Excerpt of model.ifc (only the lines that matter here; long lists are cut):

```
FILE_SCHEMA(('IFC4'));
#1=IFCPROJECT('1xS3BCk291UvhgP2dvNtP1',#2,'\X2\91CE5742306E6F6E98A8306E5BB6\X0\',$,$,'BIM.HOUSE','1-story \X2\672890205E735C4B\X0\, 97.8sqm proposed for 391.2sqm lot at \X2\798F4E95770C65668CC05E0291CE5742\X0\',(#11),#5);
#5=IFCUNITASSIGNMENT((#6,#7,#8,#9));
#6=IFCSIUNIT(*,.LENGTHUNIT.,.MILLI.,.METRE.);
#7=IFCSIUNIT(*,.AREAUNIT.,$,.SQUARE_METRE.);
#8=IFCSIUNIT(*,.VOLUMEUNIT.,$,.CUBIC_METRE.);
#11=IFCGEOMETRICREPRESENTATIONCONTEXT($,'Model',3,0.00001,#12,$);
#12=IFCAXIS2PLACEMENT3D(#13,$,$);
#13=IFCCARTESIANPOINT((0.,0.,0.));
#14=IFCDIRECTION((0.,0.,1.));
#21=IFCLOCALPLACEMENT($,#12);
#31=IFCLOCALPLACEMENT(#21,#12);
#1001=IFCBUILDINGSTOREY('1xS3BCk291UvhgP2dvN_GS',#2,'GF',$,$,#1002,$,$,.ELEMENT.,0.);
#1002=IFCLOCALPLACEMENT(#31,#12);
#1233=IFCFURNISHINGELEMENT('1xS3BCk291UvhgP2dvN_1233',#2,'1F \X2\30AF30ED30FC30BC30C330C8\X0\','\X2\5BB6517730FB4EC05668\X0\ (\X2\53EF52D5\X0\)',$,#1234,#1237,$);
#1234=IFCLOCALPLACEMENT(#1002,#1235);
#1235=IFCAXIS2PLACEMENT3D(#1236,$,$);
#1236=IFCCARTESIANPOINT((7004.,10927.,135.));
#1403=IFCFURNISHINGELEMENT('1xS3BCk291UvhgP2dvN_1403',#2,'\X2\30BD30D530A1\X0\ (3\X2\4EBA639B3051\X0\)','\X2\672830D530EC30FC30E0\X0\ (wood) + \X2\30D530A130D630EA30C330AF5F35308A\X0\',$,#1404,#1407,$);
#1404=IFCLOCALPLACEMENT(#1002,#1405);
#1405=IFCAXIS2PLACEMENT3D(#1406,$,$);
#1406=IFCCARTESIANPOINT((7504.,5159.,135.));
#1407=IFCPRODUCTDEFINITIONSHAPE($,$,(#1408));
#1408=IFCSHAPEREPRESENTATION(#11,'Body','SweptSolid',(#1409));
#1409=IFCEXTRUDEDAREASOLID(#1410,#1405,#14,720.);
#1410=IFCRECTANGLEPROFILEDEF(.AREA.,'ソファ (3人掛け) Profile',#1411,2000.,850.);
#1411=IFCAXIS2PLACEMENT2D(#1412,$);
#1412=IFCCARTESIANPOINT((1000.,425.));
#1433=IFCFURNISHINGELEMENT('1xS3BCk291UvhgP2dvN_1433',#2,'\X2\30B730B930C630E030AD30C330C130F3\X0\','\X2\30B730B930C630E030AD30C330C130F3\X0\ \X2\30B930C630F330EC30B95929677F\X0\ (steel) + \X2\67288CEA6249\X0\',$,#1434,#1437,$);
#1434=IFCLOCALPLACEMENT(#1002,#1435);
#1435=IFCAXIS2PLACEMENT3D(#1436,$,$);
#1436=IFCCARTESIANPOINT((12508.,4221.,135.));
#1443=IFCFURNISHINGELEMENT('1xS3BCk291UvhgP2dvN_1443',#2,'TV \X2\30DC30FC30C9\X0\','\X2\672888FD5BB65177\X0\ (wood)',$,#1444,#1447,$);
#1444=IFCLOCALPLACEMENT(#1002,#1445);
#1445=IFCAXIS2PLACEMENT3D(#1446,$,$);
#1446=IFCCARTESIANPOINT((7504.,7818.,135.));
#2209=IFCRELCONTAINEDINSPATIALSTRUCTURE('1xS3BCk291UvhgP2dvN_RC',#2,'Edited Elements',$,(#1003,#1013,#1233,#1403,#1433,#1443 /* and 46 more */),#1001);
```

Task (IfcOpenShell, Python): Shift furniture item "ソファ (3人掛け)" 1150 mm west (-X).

```python
import ifcopenshell
import ifcopenshell.api.geometry
import ifcopenshell.util.placement
import ifcopenshell.util.unit

model = ifcopenshell.open("model.ifc")
unit_scale = ifcopenshell.util.unit.calculate_unit_scale(model)

item = model.by_id(1403)
matrix = ifcopenshell.util.placement.get_local_placement(item.ObjectPlacement)
matrix[0, 3] -= 1.15 / unit_scale
ifcopenshell.api.geometry.edit_object_placement(model, product=item, matrix=matrix, is_si=False)

print(ifcopenshell.util.placement.get_local_placement(item.ObjectPlacement).round(3) + 0.0)

model.write("model-out.ifc")
```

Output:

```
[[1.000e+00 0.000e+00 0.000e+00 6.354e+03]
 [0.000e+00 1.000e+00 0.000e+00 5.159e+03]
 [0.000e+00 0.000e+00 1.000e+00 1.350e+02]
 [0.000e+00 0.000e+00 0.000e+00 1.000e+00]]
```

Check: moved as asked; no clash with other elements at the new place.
